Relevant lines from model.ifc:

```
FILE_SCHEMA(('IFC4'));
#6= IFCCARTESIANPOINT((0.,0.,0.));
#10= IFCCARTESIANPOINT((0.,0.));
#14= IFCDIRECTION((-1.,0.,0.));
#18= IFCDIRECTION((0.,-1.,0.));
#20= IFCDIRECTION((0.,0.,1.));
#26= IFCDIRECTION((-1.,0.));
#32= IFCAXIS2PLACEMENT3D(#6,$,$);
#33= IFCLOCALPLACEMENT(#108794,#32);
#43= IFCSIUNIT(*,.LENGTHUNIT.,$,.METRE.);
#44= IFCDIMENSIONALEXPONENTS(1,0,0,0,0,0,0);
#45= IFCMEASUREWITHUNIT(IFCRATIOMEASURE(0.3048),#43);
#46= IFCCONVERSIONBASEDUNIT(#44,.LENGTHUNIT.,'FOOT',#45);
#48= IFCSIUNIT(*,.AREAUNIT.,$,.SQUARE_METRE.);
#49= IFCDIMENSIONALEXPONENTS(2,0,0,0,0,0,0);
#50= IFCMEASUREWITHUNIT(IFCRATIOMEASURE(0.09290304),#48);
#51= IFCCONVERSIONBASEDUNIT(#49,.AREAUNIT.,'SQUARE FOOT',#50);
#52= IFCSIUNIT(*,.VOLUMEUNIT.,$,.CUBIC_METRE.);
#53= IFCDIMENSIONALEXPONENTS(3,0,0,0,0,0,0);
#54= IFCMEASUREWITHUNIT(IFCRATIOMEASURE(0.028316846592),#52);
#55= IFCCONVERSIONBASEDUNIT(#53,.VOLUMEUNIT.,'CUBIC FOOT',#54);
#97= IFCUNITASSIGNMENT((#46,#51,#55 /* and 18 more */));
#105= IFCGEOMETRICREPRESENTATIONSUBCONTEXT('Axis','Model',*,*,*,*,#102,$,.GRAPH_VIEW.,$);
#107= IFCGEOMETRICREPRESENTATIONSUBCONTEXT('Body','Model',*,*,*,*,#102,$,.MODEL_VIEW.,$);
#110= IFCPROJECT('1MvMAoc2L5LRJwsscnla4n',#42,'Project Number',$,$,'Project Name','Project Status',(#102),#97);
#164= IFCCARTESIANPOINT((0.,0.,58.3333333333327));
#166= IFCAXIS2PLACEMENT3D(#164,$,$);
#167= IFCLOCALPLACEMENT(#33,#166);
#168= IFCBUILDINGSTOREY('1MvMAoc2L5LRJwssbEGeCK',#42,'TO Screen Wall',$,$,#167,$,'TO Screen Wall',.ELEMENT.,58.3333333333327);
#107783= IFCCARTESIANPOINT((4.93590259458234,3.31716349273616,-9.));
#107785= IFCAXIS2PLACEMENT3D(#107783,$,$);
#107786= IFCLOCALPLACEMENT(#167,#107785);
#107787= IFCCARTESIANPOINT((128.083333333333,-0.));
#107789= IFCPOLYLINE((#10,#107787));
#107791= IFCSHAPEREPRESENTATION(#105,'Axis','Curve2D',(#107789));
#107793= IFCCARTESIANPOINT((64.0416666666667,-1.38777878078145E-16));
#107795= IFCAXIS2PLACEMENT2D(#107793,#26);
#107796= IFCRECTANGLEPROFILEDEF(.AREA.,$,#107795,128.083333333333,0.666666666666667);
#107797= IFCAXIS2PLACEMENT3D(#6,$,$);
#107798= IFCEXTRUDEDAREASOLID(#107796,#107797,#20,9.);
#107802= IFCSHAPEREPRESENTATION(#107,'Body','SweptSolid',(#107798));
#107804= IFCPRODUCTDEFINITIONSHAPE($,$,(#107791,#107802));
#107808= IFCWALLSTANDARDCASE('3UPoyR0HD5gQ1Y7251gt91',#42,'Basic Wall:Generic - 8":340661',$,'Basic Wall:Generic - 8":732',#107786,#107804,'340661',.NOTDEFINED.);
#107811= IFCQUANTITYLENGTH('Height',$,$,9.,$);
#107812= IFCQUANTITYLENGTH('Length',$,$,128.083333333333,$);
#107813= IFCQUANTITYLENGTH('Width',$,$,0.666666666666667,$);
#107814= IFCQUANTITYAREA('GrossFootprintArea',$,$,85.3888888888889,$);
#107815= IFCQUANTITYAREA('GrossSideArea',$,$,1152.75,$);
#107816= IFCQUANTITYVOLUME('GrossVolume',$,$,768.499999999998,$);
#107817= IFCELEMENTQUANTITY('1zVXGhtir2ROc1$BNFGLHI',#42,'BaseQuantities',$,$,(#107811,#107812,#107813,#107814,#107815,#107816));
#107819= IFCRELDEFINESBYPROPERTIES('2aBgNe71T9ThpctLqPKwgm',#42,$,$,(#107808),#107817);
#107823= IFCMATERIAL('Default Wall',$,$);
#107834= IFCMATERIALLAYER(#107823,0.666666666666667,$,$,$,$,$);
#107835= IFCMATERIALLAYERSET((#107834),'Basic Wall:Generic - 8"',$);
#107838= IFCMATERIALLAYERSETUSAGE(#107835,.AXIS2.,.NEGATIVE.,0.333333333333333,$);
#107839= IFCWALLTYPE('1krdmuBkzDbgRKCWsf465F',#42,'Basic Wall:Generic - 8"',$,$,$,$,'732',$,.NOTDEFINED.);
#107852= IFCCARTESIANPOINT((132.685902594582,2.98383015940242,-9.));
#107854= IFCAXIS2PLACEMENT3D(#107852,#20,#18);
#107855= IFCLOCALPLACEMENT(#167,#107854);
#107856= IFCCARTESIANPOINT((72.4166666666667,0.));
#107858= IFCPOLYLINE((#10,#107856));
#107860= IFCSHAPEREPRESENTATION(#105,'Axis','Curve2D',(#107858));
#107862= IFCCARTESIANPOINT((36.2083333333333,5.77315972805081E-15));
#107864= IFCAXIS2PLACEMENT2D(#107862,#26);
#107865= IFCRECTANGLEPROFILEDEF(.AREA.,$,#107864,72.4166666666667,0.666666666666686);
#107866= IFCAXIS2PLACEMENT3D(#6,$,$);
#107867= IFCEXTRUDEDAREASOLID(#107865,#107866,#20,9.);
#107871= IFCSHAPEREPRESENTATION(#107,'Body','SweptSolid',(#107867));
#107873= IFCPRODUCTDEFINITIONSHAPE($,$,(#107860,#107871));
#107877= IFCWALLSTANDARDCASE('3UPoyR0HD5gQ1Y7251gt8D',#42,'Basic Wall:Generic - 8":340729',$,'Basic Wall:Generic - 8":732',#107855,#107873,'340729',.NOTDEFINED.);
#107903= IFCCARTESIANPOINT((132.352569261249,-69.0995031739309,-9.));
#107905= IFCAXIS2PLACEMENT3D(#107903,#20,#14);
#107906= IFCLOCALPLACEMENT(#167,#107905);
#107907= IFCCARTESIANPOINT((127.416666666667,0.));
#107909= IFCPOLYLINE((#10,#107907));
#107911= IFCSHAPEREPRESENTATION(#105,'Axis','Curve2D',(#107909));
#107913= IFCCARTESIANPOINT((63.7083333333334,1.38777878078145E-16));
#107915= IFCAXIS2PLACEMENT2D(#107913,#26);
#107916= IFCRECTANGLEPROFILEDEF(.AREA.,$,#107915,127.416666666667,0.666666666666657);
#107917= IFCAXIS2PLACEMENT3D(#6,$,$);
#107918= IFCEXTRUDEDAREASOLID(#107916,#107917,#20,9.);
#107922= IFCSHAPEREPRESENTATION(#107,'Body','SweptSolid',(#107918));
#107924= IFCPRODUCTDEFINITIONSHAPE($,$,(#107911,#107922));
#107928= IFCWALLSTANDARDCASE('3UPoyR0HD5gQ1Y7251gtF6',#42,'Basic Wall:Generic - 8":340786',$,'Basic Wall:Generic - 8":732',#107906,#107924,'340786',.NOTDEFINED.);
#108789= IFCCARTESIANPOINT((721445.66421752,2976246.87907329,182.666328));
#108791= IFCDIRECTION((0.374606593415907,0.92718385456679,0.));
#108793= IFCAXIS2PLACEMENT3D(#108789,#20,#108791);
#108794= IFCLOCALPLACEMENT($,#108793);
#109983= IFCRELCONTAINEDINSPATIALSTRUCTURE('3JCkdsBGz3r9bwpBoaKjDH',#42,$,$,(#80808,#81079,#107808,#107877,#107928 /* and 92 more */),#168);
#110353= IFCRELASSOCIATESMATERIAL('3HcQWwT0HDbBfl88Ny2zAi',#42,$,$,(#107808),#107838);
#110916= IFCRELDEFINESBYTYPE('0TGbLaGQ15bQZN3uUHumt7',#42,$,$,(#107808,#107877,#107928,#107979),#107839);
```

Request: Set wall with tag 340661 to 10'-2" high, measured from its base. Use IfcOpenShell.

```python
import ifcopenshell
import ifcopenshell.api.pset
import ifcopenshell.geom
import ifcopenshell.util.element
import ifcopenshell.util.representation
import ifcopenshell.util.shape
import ifcopenshell.util.unit

model = ifcopenshell.open("model.ifc")
unit_scale = ifcopenshell.util.unit.calculate_unit_scale(model)
area_scale = ifcopenshell.util.unit.calculate_unit_scale(model, "AREAUNIT")
volume_scale = ifcopenshell.util.unit.calculate_unit_scale(model, "VOLUMEUNIT")
settings = ifcopenshell.geom.settings()


def volume(element):
    """Net volume in cubic metres, openings subtracted."""
    shape = ifcopenshell.geom.create_shape(settings, element)
    return ifcopenshell.util.shape.get_volume(shape.geometry)


wall = model.by_id(107808)
before = volume(wall)

body = ifcopenshell.util.representation.get_representation(wall, "Model", "Body")
solid = body.Items[0]
old_height = solid.Depth
solid.Depth = 122 * 0.0254 / unit_scale
after = volume(wall)

# Update the stored height, areas and volumes.
qto = model.by_id(ifcopenshell.util.element.get_pset(wall, "BaseQuantities", should_inherit=False)["id"])
ifcopenshell.api.pset.edit_qto(model, qto=qto, properties={
    "Height": solid.Depth,
    "GrossSideArea": ifcopenshell.util.element.get_pset(wall, "BaseQuantities", "GrossSideArea") * solid.Depth / old_height,
    "GrossVolume": ifcopenshell.util.element.get_pset(wall, "BaseQuantities", "GrossVolume") * solid.Depth / old_height,
})

print(f"height {old_height:g} -> {solid.Depth:g}, volume {before:.3f} -> {after:.3f} m3")

model.write("model_v2.ifc")
```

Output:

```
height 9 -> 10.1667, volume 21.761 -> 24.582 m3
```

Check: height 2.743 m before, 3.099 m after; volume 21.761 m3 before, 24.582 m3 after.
